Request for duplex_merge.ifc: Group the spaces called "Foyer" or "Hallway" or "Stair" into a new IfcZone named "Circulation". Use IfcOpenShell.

First a look at what the model holds.

```python
import ifcopenshell

model = ifcopenshell.open("duplex_merge.ifc")
print(model.schema)
seen = {}
for space in model.by_type("IfcSpace"):
    seen[space.LongName] = seen.get(space.LongName, 0) + 1
for name, count in sorted(seen.items(), key=str):
    print(count, "x", name)
print("zones:", [z.Name for z in model.by_type("IfcZone")][:20])
```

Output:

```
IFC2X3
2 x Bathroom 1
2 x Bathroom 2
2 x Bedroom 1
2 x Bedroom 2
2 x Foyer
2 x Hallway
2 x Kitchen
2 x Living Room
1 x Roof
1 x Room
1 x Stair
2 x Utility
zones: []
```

```python
import ifcopenshell
import ifcopenshell.api.group
import ifcopenshell.api.root

model = ifcopenshell.open("duplex_merge.ifc")

names = {"Foyer", "Hallway", "Stair"}
spaces = [s for s in model.by_type("IfcSpace") if s.LongName in names]

zone = ifcopenshell.api.root.create_entity(model, ifc_class="IfcZone", name="Circulation")
ifcopenshell.api.group.assign_group(model, products=spaces, group=zone)
print(len(spaces), "spaces in", zone.Name)

model.write("duplex_merge_rev.ifc")
```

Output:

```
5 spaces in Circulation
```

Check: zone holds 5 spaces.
